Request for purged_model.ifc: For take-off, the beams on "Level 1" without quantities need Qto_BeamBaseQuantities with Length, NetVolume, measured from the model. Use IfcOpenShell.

First a look at what the model holds.

```python
import ifcopenshell
import ifcopenshell.util.element
import ifcopenshell.util.unit

model = ifcopenshell.open("purged_model.ifc")
print(model.schema)
for unit_type in ("LENGTHUNIT", "AREAUNIT", "VOLUMEUNIT"):
    print(unit_type, ifcopenshell.util.unit.calculate_unit_scale(model, unit_type))
storey = next(s for s in model.by_type("IfcBuildingStorey") if s.Name == "Level 1")
beams = [e for e in ifcopenshell.util.element.get_decomposition(storey) if e.is_a("IfcBeam")]
for e in sorted(beams, key=lambda e: e.id()):
    print(e.id(), e.is_a(), e.Name, list(ifcopenshell.util.element.get_psets(e, qtos_only=True)), sep=" | ")
```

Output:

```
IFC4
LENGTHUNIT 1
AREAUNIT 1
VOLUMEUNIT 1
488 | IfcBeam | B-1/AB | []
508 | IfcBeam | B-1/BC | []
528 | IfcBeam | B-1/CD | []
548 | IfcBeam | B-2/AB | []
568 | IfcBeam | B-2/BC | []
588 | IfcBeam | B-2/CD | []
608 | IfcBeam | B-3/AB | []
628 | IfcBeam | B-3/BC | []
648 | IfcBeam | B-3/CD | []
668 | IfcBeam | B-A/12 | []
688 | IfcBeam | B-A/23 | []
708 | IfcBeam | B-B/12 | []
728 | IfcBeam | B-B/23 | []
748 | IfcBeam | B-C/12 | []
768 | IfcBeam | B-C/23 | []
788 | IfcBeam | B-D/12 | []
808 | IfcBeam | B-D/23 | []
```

```python
import ifcopenshell
import ifcopenshell.api.pset
import ifcopenshell.geom
import ifcopenshell.util.element
import ifcopenshell.util.shape
import ifcopenshell.util.unit

model = ifcopenshell.open("purged_model.ifc")
unit_scale = ifcopenshell.util.unit.calculate_unit_scale(model)
volume_scale = ifcopenshell.util.unit.calculate_unit_scale(model, "VOLUMEUNIT")
settings = ifcopenshell.geom.settings()

storey = next(s for s in model.by_type("IfcBuildingStorey") if s.Name == "Level 1")
beams = [e for e in ifcopenshell.util.element.get_decomposition(storey) if e.is_a("IfcBeam")]

for e in sorted(beams, key=lambda e: e.id()):
    if ifcopenshell.util.element.get_psets(e, qtos_only=True, should_inherit=False):
        continue
    # Geometry comes back in metres, in the element's own axes.
    shape = ifcopenshell.geom.create_shape(settings, e)
    values = {
        "Length": ifcopenshell.util.shape.get_max_xyz(shape.geometry) / unit_scale,
        "NetVolume": ifcopenshell.util.shape.get_volume(shape.geometry) / volume_scale,
    }
    qto = ifcopenshell.api.pset.add_qto(model, product=e, name="Qto_BeamBaseQuantities")
    ifcopenshell.api.pset.edit_qto(model, qto=qto, properties=values)
    print(e.id(), {k: round(v, 3) for k, v in values.items()})

model.write("purged_model_edited.ifc")
```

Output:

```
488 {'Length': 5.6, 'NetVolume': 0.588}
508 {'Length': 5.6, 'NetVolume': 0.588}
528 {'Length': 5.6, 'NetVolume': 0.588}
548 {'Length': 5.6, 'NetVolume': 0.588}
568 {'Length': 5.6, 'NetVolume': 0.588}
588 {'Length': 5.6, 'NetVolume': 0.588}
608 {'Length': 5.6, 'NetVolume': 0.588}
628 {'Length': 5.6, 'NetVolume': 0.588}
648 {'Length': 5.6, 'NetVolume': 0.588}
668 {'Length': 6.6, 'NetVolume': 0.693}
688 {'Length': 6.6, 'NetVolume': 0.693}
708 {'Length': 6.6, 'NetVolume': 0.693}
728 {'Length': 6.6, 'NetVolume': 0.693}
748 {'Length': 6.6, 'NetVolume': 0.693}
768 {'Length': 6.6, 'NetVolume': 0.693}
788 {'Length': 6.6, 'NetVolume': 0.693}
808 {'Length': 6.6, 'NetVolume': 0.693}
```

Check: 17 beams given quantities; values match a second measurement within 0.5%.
